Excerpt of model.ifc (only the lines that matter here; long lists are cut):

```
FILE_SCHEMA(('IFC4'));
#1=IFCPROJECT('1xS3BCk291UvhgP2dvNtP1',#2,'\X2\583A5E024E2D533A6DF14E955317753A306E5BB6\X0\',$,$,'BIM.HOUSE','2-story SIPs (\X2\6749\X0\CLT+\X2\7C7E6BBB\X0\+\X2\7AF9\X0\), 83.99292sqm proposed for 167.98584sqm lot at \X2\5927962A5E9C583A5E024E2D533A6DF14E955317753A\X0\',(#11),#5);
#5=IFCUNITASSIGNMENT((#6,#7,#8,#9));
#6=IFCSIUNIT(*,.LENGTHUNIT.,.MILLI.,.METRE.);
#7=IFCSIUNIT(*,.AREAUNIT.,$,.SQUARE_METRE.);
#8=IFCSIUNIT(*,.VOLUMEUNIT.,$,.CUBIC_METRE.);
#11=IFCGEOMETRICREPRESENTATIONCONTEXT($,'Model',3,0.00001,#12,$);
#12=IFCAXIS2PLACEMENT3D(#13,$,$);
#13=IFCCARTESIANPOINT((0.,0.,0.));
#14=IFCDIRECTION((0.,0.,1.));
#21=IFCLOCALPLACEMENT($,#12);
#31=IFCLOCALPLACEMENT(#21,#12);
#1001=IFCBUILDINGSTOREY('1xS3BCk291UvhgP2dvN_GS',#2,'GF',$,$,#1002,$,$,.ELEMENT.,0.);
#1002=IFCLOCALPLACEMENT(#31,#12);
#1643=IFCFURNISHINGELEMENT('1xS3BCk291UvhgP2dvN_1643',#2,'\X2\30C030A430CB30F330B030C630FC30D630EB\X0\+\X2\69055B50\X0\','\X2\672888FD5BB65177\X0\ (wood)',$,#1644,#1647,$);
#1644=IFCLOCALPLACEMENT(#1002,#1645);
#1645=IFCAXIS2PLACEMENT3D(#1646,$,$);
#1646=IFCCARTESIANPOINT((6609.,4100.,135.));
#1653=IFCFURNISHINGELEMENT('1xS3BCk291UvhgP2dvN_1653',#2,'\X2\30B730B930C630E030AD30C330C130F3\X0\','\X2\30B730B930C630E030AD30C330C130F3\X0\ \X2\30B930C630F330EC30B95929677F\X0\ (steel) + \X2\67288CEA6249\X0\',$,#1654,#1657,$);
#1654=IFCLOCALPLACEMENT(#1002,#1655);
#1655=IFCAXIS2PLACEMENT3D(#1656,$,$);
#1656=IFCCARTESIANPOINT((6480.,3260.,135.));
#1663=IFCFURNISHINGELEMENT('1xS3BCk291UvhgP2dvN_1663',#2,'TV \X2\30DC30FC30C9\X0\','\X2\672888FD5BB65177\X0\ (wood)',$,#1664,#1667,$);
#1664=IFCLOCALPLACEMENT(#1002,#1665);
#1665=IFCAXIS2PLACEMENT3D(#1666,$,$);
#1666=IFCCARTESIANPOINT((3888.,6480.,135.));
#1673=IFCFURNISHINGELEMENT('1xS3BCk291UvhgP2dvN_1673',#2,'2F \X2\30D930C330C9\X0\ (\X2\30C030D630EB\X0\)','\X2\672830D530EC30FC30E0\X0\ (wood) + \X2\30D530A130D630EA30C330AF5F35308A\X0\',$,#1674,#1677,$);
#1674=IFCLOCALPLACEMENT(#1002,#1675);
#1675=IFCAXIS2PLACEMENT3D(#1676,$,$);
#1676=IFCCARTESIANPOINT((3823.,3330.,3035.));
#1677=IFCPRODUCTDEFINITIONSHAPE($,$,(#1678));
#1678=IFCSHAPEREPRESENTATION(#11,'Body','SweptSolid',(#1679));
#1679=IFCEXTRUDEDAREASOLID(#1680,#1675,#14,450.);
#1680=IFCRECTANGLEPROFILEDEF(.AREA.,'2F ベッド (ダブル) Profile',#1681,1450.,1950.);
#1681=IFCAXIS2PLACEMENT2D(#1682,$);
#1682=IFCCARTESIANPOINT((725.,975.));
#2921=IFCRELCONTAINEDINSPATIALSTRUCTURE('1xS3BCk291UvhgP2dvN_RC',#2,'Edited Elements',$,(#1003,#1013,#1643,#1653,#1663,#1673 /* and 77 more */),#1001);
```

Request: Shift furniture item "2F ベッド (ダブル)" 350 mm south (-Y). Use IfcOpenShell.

```python
import ifcopenshell
import ifcopenshell.api.geometry
import ifcopenshell.util.placement
import ifcopenshell.util.unit

model = ifcopenshell.open("model.ifc")
unit_scale = ifcopenshell.util.unit.calculate_unit_scale(model)

item = model.by_guid("1xS3BCk291UvhgP2dvN_1673")
matrix = ifcopenshell.util.placement.get_local_placement(item.ObjectPlacement)
matrix[1, 3] -= 0.35 / unit_scale
ifcopenshell.api.geometry.edit_object_placement(model, product=item, matrix=matrix, is_si=False)

print(ifcopenshell.util.placement.get_local_placement(item.ObjectPlacement).round(3) + 0.0)

model.write("model-out.ifc")
```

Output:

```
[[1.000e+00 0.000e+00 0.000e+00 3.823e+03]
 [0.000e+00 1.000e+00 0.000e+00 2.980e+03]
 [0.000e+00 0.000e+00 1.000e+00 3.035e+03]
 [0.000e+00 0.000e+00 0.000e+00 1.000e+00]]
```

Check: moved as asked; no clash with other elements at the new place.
